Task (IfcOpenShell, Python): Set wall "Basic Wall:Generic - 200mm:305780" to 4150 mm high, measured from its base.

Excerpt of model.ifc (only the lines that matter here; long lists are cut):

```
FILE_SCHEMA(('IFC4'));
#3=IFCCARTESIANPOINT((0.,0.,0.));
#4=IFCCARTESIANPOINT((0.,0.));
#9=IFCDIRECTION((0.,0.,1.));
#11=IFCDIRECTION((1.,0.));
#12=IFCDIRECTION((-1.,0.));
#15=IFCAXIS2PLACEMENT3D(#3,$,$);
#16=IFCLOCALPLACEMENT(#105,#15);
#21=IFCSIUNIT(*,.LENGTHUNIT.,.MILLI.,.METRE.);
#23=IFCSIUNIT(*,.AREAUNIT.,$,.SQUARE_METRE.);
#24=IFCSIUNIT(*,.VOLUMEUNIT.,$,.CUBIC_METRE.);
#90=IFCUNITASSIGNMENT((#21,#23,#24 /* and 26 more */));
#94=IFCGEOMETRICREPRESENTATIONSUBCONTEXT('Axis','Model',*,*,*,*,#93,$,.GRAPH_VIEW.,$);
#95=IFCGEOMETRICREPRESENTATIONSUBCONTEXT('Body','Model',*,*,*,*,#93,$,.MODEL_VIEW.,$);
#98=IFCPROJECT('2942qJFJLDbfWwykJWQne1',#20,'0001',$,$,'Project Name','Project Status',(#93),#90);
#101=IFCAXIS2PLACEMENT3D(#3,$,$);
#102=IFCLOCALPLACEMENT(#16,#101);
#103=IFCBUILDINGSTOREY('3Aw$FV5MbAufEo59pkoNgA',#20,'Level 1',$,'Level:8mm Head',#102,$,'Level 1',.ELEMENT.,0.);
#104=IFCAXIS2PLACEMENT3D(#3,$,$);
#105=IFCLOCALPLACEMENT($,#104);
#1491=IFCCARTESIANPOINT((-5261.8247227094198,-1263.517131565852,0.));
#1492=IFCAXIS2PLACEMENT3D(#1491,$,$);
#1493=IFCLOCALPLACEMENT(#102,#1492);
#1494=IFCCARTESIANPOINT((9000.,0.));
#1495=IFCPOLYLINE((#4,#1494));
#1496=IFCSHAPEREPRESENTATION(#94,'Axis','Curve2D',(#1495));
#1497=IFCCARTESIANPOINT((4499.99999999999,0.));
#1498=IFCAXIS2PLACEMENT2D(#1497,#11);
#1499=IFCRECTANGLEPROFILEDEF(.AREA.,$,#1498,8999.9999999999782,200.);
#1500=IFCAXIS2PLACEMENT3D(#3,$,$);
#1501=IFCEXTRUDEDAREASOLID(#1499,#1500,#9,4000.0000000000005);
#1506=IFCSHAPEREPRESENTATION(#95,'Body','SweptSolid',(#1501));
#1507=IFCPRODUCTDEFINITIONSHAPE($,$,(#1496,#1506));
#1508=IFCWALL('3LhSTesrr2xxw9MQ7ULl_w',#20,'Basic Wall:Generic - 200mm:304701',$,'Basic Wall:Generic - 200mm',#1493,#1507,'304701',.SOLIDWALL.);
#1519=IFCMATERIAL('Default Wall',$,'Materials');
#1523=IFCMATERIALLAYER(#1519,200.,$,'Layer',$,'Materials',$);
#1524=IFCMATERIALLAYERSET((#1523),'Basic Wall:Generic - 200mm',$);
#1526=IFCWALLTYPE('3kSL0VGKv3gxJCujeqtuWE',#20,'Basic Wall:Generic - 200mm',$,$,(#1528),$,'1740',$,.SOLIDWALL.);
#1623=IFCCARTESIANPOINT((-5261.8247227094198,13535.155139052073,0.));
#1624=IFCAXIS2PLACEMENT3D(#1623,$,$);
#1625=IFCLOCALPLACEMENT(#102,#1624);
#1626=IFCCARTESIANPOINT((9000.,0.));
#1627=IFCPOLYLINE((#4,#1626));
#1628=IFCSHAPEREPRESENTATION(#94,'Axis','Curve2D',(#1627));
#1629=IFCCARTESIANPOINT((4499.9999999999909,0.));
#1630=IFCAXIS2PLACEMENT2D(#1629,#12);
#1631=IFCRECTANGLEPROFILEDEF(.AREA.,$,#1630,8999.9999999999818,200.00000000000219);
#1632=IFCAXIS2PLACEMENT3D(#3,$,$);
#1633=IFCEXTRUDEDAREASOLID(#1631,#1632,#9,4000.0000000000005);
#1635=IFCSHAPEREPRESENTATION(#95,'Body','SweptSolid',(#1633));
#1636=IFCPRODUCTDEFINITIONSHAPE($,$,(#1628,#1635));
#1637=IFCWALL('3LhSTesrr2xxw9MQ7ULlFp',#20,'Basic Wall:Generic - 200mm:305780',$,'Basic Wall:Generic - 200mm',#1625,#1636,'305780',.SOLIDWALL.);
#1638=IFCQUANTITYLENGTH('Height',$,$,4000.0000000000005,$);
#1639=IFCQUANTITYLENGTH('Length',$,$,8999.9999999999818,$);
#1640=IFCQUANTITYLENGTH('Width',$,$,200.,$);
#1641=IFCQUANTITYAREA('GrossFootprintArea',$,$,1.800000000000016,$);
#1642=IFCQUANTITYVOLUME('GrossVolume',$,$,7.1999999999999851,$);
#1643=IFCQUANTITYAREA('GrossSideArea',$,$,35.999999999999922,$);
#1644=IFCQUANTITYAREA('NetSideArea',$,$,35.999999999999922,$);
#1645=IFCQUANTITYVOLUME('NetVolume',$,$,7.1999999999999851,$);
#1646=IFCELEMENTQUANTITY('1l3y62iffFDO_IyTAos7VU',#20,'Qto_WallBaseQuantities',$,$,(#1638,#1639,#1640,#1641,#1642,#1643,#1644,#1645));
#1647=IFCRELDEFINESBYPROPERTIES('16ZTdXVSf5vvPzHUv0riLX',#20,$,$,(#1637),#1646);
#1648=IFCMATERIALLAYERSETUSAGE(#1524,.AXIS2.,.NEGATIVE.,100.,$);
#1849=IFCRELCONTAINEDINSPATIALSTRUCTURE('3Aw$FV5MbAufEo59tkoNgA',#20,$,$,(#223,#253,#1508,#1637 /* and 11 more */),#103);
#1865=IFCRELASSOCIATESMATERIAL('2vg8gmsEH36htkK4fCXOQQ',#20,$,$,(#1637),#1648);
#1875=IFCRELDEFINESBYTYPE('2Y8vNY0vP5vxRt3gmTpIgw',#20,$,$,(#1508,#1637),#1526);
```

```python
import ifcopenshell
import ifcopenshell.api.pset
import ifcopenshell.geom
import ifcopenshell.util.element
import ifcopenshell.util.representation
import ifcopenshell.util.shape
import ifcopenshell.util.unit

model = ifcopenshell.open("model.ifc")
unit_scale = ifcopenshell.util.unit.calculate_unit_scale(model)
area_scale = ifcopenshell.util.unit.calculate_unit_scale(model, "AREAUNIT")
volume_scale = ifcopenshell.util.unit.calculate_unit_scale(model, "VOLUMEUNIT")
settings = ifcopenshell.geom.settings()


def volume(element):
    """Net volume in cubic metres, openings subtracted."""
    shape = ifcopenshell.geom.create_shape(settings, element)
    return ifcopenshell.util.shape.get_volume(shape.geometry)


wall = model.by_guid("3LhSTesrr2xxw9MQ7ULlFp")
before = volume(wall)

body = ifcopenshell.util.representation.get_representation(wall, "Model", "Body")
solid = body.Items[0]
old_height = solid.Depth
solid.Depth = 4.15 / unit_scale
after = volume(wall)
thickness = 0.2  # wall thickness in metres

# Update the stored height, areas and volumes.
qto = model.by_id(ifcopenshell.util.element.get_pset(wall, "Qto_WallBaseQuantities", should_inherit=False)["id"])
ifcopenshell.api.pset.edit_qto(model, qto=qto, properties={
    "Height": solid.Depth,
    "GrossVolume": ifcopenshell.util.element.get_pset(wall, "Qto_WallBaseQuantities", "GrossVolume") * solid.Depth / old_height,
    "GrossSideArea": ifcopenshell.util.element.get_pset(wall, "Qto_WallBaseQuantities", "GrossSideArea") * solid.Depth / old_height,
    "NetSideArea": after / thickness / area_scale,
    "NetVolume": after / volume_scale,
})

print(f"height {old_height:g} -> {solid.Depth:g}, volume {before:.3f} -> {after:.3f} m3")

model.write("model_updated.ifc")
```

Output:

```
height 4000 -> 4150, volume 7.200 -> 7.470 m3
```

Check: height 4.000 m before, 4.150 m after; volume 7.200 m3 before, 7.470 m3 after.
